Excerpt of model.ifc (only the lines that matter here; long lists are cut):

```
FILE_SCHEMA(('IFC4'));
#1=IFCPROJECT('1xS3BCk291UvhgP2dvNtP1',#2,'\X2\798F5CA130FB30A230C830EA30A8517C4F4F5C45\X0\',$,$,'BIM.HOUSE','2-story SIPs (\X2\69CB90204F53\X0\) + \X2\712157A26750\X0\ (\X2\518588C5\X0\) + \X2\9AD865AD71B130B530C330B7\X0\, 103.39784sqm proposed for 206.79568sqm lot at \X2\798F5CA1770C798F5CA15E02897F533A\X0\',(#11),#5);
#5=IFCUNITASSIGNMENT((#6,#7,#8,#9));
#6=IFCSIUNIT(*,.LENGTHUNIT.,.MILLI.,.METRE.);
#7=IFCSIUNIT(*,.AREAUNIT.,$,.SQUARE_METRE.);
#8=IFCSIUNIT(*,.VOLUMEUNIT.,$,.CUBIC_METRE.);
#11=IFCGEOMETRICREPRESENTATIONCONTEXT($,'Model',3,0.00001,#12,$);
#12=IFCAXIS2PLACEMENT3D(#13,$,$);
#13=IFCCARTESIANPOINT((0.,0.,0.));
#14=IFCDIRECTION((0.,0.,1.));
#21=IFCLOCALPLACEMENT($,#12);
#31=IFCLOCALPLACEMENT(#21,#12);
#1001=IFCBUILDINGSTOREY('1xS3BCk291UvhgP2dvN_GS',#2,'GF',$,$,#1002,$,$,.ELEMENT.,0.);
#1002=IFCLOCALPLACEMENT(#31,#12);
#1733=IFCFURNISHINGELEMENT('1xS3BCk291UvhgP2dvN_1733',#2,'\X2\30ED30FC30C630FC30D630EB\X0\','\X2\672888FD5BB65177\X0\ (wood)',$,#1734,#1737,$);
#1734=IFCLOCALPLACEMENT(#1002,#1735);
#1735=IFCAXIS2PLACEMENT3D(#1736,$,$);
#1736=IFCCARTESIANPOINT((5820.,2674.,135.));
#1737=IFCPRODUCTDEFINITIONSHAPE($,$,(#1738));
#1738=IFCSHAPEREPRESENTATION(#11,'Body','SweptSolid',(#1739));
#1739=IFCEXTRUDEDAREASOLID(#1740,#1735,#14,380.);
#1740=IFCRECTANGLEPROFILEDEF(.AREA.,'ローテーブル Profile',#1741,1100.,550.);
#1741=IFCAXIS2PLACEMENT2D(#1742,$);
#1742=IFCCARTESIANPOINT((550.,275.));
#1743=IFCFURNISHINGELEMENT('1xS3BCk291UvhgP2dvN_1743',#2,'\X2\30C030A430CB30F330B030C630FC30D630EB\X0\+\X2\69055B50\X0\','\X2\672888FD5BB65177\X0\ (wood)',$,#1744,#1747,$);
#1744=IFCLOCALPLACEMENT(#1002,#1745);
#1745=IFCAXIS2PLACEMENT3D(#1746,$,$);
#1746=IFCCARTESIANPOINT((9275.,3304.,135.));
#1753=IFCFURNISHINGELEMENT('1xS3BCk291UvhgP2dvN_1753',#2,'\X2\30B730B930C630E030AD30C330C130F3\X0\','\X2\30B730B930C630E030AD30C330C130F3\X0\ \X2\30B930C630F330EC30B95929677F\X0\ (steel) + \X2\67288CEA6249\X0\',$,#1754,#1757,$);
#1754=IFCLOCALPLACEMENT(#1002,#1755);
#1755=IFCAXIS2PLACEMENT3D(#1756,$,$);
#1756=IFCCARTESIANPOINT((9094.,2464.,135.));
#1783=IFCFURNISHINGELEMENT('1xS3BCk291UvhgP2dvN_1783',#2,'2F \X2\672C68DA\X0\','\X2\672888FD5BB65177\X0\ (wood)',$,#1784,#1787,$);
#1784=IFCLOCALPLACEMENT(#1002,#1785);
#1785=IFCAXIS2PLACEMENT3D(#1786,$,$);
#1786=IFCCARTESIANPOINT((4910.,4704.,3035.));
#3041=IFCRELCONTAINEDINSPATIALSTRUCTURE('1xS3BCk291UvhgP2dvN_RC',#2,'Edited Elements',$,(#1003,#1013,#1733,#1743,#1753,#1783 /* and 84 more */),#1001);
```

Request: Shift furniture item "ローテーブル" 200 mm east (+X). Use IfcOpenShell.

```python
import ifcopenshell
import ifcopenshell.api.geometry
import ifcopenshell.util.placement

model = ifcopenshell.open("model.ifc")

item = model.by_guid("1xS3BCk291UvhgP2dvN_1733")
matrix = ifcopenshell.util.placement.get_local_placement(item.ObjectPlacement)
matrix[0, 3] += 200.0
ifcopenshell.api.geometry.edit_object_placement(model, product=item, matrix=matrix, is_si=False)

print(ifcopenshell.util.placement.get_local_placement(item.ObjectPlacement).round(3) + 0.0)

model.write("model_rev.ifc")
```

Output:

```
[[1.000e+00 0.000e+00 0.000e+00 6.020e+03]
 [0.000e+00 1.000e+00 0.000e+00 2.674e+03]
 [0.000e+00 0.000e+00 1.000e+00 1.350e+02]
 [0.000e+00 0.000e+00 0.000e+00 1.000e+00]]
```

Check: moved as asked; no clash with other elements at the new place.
